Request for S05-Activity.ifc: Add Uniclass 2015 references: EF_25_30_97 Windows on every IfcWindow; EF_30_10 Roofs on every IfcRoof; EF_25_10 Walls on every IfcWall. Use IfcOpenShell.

First a look at what the model holds.

```python
import ifcopenshell

model = ifcopenshell.open("S05-Activity.ifc")
print(model.schema)
print("classifications:", [c.Name for c in model.by_type("IfcClassification")])
for ifc_class in ("IfcDoor", "IfcRoof", "IfcStair", "IfcWall", "IfcWindow"):
    print(ifc_class, len(model.by_type(ifc_class)))
```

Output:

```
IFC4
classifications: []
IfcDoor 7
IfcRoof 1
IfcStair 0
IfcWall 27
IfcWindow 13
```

```python
import ifcopenshell
import ifcopenshell.api.classification

model = ifcopenshell.open("S05-Activity.ifc")

system = ifcopenshell.api.classification.add_classification(model, classification="Uniclass 2015")

codes = {
    "IfcWindow": ("EF_25_30_97", "Windows"),
    "IfcRoof": ("EF_30_10", "Roofs"),
    "IfcWall": ("EF_25_10", "Walls"),
}
for ifc_class, (code, name) in codes.items():
    products = model.by_type(ifc_class)
    ifcopenshell.api.classification.add_reference(
        model, products=products, classification=system, identification=code, name=name
    )
    print(code, len(products))

model.write("S05-Activity_v2.ifc")
```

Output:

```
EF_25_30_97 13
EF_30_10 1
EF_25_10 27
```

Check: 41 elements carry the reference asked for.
